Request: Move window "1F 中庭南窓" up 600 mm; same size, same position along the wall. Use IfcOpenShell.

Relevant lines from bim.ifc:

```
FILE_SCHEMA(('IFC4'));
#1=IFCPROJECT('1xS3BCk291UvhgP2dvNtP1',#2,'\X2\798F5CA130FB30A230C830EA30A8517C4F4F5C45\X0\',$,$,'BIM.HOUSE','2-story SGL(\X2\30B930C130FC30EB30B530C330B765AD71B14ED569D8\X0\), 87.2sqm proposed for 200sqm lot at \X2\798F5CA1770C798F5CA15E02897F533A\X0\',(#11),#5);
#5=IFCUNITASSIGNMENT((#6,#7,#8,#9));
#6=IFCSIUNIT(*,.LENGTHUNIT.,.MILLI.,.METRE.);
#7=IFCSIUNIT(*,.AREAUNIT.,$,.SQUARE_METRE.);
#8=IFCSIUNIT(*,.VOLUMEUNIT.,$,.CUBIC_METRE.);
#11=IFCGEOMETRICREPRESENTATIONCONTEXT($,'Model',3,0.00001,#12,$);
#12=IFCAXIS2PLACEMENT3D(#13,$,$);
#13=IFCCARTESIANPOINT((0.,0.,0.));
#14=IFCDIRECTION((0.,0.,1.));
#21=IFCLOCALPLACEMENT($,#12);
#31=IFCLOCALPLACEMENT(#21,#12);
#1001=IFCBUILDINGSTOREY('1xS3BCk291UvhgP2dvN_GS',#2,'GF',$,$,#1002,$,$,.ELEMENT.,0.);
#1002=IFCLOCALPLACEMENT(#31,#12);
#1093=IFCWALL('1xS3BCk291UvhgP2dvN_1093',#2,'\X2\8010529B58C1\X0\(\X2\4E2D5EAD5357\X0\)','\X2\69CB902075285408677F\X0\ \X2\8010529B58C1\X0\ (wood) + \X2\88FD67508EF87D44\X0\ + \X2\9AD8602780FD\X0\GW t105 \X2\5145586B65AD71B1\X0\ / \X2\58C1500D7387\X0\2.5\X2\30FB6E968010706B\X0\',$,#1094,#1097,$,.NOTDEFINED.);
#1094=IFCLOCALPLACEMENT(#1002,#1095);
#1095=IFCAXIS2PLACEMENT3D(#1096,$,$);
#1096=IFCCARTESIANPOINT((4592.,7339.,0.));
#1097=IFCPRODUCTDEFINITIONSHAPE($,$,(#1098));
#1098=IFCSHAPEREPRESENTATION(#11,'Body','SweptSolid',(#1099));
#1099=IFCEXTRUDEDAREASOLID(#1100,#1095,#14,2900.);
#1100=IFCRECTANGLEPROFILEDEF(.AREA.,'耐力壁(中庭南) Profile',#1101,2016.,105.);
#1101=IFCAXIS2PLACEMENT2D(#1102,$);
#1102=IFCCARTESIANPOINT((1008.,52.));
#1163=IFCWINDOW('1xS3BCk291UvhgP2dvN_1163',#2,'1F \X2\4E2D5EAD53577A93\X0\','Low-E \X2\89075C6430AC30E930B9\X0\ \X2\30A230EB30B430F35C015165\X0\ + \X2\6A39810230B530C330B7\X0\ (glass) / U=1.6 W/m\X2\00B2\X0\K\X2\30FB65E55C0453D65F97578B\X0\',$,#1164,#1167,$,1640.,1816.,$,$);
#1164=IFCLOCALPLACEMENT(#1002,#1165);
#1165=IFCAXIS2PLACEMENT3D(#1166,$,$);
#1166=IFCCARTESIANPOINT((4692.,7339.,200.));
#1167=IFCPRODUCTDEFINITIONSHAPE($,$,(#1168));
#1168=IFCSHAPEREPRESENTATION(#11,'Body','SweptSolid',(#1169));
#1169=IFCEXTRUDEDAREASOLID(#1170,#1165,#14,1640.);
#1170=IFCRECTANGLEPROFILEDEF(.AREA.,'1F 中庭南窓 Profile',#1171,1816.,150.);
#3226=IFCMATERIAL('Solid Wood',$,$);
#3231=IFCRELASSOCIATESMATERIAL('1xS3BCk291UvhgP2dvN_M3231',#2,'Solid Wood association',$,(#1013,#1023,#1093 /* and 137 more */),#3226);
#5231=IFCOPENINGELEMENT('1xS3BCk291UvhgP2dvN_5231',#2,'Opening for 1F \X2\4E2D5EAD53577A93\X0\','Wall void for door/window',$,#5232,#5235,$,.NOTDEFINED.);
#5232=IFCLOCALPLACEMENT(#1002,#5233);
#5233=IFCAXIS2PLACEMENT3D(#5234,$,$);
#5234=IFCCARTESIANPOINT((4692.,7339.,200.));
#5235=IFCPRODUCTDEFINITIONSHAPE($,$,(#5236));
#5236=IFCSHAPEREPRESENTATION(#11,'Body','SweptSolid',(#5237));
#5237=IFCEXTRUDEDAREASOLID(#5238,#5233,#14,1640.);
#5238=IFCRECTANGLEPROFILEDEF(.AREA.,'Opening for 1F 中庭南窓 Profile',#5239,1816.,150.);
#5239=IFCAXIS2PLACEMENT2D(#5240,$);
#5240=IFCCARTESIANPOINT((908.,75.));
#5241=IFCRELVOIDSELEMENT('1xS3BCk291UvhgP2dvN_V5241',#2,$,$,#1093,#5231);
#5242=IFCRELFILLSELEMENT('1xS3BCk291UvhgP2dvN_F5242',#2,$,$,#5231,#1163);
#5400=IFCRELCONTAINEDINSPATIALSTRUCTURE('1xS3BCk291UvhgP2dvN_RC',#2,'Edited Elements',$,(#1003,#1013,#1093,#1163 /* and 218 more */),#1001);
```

```python
import numpy as np
import ifcopenshell
import ifcopenshell.api.geometry
import ifcopenshell.util.placement
import ifcopenshell.util.unit

model = ifcopenshell.open("bim.ifc")
unit_scale = ifcopenshell.util.unit.calculate_unit_scale(model)

window = model.by_guid("1xS3BCk291UvhgP2dvN_1163")
opening = window.FillsVoids[0].RelatingOpeningElement
dz = 0.6 / unit_scale

shift = np.array([0.0, 0.0, dz])
# The window is not placed relative to its opening, so move both.
for product in (opening, window):
    matrix = ifcopenshell.util.placement.get_local_placement(product.ObjectPlacement)
    matrix[:3, 3] += shift
    ifcopenshell.api.geometry.edit_object_placement(model, product=product, matrix=matrix, is_si=False)

print(f"moved by {dz * unit_scale:+.3f} m")

model.write("bim_v2.ifc")
```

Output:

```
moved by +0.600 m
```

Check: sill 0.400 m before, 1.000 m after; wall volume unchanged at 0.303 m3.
